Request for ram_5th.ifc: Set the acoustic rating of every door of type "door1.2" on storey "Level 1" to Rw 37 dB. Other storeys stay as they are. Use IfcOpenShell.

First a look at what the model holds.

```python
import ifcopenshell
import ifcopenshell.util.element

model = ifcopenshell.open("ram_5th.ifc")
print(model.schema)
storey = next(s for s in model.by_type("IfcBuildingStorey") if s.Name == "Level 1")
doors = [e for e in ifcopenshell.util.element.get_decomposition(storey) if e.is_a("IfcDoor")]
seen = {}
for e in doors:
    element_type = ifcopenshell.util.element.get_type(e)
    key = (element_type.Name if element_type != e and element_type else None, ifcopenshell.util.element.get_pset(e, "Pset_DoorCommon", "AcousticRating"))
    seen[key] = seen.get(key, 0) + 1
for (name, value), count in sorted(seen.items(), key=str):
    print(count, "x", name, "|", value)
```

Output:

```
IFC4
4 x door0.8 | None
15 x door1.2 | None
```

```python
import ifcopenshell
import ifcopenshell.api.pset
import ifcopenshell.util.element

model = ifcopenshell.open("ram_5th.ifc")

storey = next(s for s in model.by_type("IfcBuildingStorey") if s.Name == "Level 1")
doors = [e for e in ifcopenshell.util.element.get_decomposition(storey) if e.is_a("IfcDoor")]

count = 0
for e in doors:
    element_type = ifcopenshell.util.element.get_type(e)
    if element_type in (None, e) or element_type.Name != "door1.2":
        continue
    # add_pset returns the element's existing set when there is one.
    pset = ifcopenshell.api.pset.add_pset(model, product=e, name="Pset_DoorCommon")
    ifcopenshell.api.pset.edit_pset(model, pset=pset, properties={"AcousticRating": "Rw 37 dB"})
    count += 1

print(count, "doors updated")

model.write("ram_5th_rev.ifc")
```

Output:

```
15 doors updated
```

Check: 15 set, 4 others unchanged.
